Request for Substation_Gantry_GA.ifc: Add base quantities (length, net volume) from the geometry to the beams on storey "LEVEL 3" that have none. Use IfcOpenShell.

First a look at what the model holds.

```python
import ifcopenshell
import ifcopenshell.util.element
import ifcopenshell.util.unit

model = ifcopenshell.open("Substation_Gantry_GA.ifc")
print(model.schema)
for unit_type in ("LENGTHUNIT", "AREAUNIT", "VOLUMEUNIT"):
    print(unit_type, ifcopenshell.util.unit.calculate_unit_scale(model, unit_type))
storey = next(s for s in model.by_type("IfcBuildingStorey") if s.Name == "LEVEL 3")
beams = [e for e in ifcopenshell.util.element.get_decomposition(storey) if e.is_a("IfcBeam")]
for e in sorted(beams, key=lambda e: e.id()):
    print(e.id(), e.is_a(), e.Name, list(ifcopenshell.util.element.get_psets(e, qtos_only=True)), sep=" | ")
```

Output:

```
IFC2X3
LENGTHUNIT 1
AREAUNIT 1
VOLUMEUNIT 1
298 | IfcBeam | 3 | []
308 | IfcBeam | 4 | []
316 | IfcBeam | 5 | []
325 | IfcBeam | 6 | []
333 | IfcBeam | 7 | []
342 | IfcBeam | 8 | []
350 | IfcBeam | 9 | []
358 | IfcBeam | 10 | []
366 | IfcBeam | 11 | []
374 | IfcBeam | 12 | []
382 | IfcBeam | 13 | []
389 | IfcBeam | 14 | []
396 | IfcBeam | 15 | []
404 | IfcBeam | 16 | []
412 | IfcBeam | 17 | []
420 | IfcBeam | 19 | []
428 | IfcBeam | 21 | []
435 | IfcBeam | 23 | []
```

```python
import ifcopenshell
import ifcopenshell.api.pset
import ifcopenshell.geom
import ifcopenshell.util.element
import ifcopenshell.util.shape
import ifcopenshell.util.unit

model = ifcopenshell.open("Substation_Gantry_GA.ifc")
unit_scale = ifcopenshell.util.unit.calculate_unit_scale(model)
volume_scale = ifcopenshell.util.unit.calculate_unit_scale(model, "VOLUMEUNIT")
settings = ifcopenshell.geom.settings()

storey = next(s for s in model.by_type("IfcBuildingStorey") if s.Name == "LEVEL 3")
beams = [e for e in ifcopenshell.util.element.get_decomposition(storey) if e.is_a("IfcBeam")]

for e in sorted(beams, key=lambda e: e.id()):
    if ifcopenshell.util.element.get_psets(e, qtos_only=True, should_inherit=False):
        continue
    # Geometry comes back in metres, in the element's own axes.
    shape = ifcopenshell.geom.create_shape(settings, e)
    values = {
        "Length": ifcopenshell.util.shape.get_max_xyz(shape.geometry) / unit_scale,
        "NetVolume": ifcopenshell.util.shape.get_volume(shape.geometry) / volume_scale,
    }
    qto = ifcopenshell.api.pset.add_qto(model, product=e, name="BaseQuantities")
    ifcopenshell.api.pset.edit_qto(model, qto=qto, properties=values)
    print(e.id(), {k: round(v, 3) for k, v in values.items()})

model.write("Substation_Gantry_GA_rev.ifc")
```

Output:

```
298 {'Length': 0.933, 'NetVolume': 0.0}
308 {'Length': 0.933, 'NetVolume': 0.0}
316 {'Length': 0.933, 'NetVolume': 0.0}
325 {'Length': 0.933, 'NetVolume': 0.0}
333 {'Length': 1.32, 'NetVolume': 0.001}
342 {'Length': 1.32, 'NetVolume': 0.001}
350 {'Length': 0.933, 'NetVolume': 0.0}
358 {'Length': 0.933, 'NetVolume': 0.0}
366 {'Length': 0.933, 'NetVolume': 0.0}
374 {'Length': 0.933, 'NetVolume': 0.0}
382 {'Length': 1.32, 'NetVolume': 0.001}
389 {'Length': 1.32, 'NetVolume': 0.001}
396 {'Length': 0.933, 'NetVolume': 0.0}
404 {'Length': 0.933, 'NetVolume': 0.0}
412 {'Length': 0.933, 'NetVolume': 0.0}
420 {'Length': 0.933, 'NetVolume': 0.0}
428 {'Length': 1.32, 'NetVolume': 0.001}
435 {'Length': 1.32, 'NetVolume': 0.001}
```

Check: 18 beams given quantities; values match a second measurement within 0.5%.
